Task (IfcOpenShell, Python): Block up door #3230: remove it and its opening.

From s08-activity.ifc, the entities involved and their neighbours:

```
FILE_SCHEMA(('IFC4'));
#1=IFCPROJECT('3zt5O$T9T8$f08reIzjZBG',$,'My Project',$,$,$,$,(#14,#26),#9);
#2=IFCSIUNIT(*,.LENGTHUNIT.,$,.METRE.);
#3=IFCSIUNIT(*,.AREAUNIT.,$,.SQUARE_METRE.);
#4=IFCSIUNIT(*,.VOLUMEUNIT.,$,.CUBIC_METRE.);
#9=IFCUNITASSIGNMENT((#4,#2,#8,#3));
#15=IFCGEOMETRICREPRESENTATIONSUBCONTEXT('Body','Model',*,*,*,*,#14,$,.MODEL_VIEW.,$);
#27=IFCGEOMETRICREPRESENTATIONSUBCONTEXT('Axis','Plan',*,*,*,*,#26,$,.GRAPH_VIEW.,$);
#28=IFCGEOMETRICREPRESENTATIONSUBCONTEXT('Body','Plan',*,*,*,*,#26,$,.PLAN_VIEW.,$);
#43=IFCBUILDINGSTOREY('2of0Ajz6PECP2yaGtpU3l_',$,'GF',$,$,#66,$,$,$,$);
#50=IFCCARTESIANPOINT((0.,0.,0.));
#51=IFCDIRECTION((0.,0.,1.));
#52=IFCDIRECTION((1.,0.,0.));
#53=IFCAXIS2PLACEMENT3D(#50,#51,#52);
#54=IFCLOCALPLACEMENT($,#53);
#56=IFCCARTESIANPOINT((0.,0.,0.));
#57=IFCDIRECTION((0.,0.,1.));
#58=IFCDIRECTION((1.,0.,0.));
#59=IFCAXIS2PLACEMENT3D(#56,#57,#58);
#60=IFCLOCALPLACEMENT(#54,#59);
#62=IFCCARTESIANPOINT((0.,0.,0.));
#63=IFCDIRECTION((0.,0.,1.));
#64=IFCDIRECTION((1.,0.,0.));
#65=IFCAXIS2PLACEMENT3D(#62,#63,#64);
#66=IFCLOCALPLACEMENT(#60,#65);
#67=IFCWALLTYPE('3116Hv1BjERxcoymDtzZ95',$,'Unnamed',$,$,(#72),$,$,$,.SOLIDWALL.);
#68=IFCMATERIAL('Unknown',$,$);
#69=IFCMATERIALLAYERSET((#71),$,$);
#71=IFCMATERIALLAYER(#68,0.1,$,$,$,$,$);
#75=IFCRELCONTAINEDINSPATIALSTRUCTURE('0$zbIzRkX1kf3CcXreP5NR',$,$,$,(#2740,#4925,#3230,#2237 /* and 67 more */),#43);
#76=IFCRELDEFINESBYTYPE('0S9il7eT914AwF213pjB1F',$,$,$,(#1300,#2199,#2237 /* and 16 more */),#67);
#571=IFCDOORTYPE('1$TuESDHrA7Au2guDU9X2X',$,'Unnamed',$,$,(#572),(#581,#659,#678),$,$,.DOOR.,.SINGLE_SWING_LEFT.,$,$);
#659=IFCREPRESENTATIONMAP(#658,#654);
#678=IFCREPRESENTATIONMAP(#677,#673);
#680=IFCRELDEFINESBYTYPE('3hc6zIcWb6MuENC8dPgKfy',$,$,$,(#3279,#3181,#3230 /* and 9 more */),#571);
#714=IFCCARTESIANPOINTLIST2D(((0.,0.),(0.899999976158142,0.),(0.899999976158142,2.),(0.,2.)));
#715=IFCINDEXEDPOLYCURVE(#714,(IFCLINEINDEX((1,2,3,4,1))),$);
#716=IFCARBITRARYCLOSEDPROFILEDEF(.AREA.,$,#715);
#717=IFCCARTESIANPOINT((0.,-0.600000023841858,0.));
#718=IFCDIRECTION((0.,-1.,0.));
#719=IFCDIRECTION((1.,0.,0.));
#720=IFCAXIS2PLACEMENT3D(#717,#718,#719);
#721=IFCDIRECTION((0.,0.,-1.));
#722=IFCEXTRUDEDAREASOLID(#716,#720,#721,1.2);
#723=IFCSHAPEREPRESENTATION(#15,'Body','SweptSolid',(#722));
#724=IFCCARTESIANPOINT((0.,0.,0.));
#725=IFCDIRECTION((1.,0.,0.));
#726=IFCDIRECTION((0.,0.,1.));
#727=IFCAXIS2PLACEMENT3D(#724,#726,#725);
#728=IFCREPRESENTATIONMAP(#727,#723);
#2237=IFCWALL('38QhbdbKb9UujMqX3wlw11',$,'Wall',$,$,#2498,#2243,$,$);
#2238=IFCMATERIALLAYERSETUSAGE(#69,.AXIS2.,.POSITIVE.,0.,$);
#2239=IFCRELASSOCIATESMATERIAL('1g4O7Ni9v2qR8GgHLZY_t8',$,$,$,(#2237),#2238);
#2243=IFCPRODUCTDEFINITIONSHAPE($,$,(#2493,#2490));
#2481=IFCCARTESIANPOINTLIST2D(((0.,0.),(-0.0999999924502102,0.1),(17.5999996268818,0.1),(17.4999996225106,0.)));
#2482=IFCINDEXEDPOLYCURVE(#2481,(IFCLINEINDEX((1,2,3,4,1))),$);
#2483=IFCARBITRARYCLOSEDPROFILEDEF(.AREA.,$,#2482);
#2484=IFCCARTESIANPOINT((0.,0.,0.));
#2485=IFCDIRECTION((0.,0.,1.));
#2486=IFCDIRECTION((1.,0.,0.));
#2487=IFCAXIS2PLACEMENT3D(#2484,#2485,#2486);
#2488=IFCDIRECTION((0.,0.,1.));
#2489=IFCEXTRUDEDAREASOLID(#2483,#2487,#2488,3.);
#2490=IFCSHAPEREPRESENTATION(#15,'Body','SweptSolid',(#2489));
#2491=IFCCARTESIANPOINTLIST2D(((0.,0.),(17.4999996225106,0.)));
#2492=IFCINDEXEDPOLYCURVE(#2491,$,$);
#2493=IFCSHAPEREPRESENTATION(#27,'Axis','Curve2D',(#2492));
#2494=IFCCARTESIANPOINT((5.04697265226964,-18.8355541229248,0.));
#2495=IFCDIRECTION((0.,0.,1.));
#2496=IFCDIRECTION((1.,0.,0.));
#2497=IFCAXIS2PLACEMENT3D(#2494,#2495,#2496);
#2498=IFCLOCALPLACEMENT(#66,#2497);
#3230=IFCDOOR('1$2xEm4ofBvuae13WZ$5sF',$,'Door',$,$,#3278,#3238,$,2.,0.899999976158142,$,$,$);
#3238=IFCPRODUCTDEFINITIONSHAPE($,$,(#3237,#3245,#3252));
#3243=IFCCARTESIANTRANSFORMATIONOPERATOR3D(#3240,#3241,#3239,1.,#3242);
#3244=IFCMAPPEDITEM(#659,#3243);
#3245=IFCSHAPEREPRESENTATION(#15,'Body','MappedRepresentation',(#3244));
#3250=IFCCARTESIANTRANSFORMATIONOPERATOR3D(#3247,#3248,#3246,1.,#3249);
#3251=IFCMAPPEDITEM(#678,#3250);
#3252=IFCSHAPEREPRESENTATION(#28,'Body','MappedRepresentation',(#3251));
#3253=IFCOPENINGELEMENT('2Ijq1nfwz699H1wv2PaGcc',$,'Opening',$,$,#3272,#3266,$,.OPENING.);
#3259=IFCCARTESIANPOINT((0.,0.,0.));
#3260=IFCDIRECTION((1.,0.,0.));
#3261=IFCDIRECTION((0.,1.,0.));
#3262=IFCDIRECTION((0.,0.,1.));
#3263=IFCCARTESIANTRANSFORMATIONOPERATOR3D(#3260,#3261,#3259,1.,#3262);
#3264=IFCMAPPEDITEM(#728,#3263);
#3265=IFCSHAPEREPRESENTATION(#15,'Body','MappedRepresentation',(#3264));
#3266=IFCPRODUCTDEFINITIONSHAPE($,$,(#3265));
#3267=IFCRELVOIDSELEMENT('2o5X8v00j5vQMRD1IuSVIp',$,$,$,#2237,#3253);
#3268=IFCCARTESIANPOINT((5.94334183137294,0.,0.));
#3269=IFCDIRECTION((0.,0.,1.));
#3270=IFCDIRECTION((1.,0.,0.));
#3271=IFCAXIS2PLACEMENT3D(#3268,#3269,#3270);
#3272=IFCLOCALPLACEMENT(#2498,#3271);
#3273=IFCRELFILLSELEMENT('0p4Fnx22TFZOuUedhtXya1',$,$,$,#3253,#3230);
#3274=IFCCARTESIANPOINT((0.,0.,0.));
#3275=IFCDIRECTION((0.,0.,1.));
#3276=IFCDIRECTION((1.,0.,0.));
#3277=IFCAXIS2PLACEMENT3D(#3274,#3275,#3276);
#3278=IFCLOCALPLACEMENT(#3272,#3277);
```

```python
import ifcopenshell
import ifcopenshell.api.feature
import ifcopenshell.api.root
import ifcopenshell.geom
import ifcopenshell.util.shape

model = ifcopenshell.open("s08-activity.ifc")
settings = ifcopenshell.geom.settings()


def volume(element):
    """Net volume in cubic metres, openings subtracted."""
    shape = ifcopenshell.geom.create_shape(settings, element)
    return ifcopenshell.util.shape.get_volume(shape.geometry)


door = model.by_id(3230)
opening = door.FillsVoids[0].RelatingOpeningElement
wall = opening.VoidsElements[0].RelatingBuildingElement
before = volume(wall)

ifcopenshell.api.root.remove_product(model, product=door)
ifcopenshell.api.feature.remove_feature(model, feature=opening)

after = volume(wall)

print(f"wall volume {before:.3f} -> {after:.3f} m3")

model.write("s08-activity_edited.ifc")
```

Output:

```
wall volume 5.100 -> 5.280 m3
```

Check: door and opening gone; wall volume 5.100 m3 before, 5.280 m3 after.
